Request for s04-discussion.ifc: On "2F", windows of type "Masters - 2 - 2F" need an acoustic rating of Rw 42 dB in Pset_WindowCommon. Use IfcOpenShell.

First a look at what the model holds.

```python
import ifcopenshell
import ifcopenshell.util.element

model = ifcopenshell.open("s04-discussion.ifc")
print(model.schema)
storey = next(s for s in model.by_type("IfcBuildingStorey") if s.Name == "2F")
windows = [e for e in ifcopenshell.util.element.get_decomposition(storey) if e.is_a("IfcWindow")]
seen = {}
for e in windows:
    element_type = ifcopenshell.util.element.get_type(e)
    key = (element_type.Name if element_type != e and element_type else None, ifcopenshell.util.element.get_pset(e, "Pset_WindowCommon", "AcousticRating"))
    seen[key] = seen.get(key, 0) + 1
for (name, value), count in sorted(seen.items(), key=str):
    print(count, "x", name, "|", value)
```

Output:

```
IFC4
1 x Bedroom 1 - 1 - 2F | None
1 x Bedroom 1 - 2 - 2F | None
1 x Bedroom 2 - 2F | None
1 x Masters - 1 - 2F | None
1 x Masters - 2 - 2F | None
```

```python
import ifcopenshell
import ifcopenshell.api.pset
import ifcopenshell.util.element

model = ifcopenshell.open("s04-discussion.ifc")

storey = next(s for s in model.by_type("IfcBuildingStorey") if s.Name == "2F")
windows = [e for e in ifcopenshell.util.element.get_decomposition(storey) if e.is_a("IfcWindow")]

count = 0
for e in windows:
    element_type = ifcopenshell.util.element.get_type(e)
    if element_type in (None, e) or element_type.Name != "Masters - 2 - 2F":
        continue
    # add_pset returns the element's existing set when there is one.
    pset = ifcopenshell.api.pset.add_pset(model, product=e, name="Pset_WindowCommon")
    ifcopenshell.api.pset.edit_pset(model, pset=pset, properties={"AcousticRating": "Rw 42 dB"})
    count += 1

print(count, "windows updated")

model.write("s04-discussion_edited.ifc")
```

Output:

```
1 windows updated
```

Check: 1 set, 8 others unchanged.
